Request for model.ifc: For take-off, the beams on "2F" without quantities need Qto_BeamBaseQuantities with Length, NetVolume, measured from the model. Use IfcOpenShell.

First a look at what the model holds.

```python
import ifcopenshell
import ifcopenshell.util.element
import ifcopenshell.util.unit

model = ifcopenshell.open("model.ifc")
print(model.schema)
for unit_type in ("LENGTHUNIT", "AREAUNIT", "VOLUMEUNIT"):
    print(unit_type, ifcopenshell.util.unit.calculate_unit_scale(model, unit_type))
storey = next(s for s in model.by_type("IfcBuildingStorey") if s.Name == "2F")
beams = [e for e in ifcopenshell.util.element.get_decomposition(storey) if e.is_a("IfcBeam")]
for e in sorted(beams, key=lambda e: e.id()):
    print(e.id(), e.is_a(), e.Name, list(ifcopenshell.util.element.get_psets(e, qtos_only=True)), sep=" | ")
```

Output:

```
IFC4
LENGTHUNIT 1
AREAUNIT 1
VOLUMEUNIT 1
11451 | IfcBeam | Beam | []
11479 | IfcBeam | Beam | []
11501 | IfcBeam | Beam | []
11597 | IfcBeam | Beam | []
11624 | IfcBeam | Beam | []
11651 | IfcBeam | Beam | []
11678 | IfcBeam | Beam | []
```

```python
import ifcopenshell
import ifcopenshell.api.pset
import ifcopenshell.geom
import ifcopenshell.util.element
import ifcopenshell.util.shape
import ifcopenshell.util.unit

model = ifcopenshell.open("model.ifc")
unit_scale = ifcopenshell.util.unit.calculate_unit_scale(model)
volume_scale = ifcopenshell.util.unit.calculate_unit_scale(model, "VOLUMEUNIT")
settings = ifcopenshell.geom.settings()

storey = next(s for s in model.by_type("IfcBuildingStorey") if s.Name == "2F")
beams = [e for e in ifcopenshell.util.element.get_decomposition(storey) if e.is_a("IfcBeam")]

for e in sorted(beams, key=lambda e: e.id()):
    if ifcopenshell.util.element.get_psets(e, qtos_only=True, should_inherit=False):
        continue
    # Geometry comes back in metres, in the element's own axes.
    shape = ifcopenshell.geom.create_shape(settings, e)
    values = {
        "Length": ifcopenshell.util.shape.get_max_xyz(shape.geometry) / unit_scale,
        "NetVolume": ifcopenshell.util.shape.get_volume(shape.geometry) / volume_scale,
    }
    qto = ifcopenshell.api.pset.add_qto(model, product=e, name="Qto_BeamBaseQuantities")
    ifcopenshell.api.pset.edit_qto(model, qto=qto, properties=values)
    print(e.id(), {k: round(v, 3) for k, v in values.items()})

model.write("model_updated.ifc")
```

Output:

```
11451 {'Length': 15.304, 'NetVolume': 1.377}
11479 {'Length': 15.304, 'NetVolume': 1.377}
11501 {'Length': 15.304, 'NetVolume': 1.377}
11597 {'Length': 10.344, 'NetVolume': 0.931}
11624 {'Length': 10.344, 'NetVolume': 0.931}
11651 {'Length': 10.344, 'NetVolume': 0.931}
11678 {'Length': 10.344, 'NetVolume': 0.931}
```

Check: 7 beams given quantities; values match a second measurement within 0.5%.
